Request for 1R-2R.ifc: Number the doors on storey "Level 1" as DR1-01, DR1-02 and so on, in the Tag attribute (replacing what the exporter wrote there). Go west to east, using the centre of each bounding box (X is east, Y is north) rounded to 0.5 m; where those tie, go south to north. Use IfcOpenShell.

First a look at what the model holds.

```python
import ifcopenshell
import ifcopenshell.util.element
import ifcopenshell.util.placement

model = ifcopenshell.open("1R-2R.ifc")
print(model.schema)
storey = next(s for s in model.by_type("IfcBuildingStorey") if s.Name == "Level 1")
doors = [e for e in ifcopenshell.util.element.get_decomposition(storey) if e.is_a("IfcDoor")]
for e in sorted(doors, key=lambda e: e.id()):
    origin = ifcopenshell.util.placement.get_local_placement(e.ObjectPlacement)[:3, 3]
    print(e.id(), e.Tag, e.Name, origin.round(2) + 0.0, sep=" | ")
```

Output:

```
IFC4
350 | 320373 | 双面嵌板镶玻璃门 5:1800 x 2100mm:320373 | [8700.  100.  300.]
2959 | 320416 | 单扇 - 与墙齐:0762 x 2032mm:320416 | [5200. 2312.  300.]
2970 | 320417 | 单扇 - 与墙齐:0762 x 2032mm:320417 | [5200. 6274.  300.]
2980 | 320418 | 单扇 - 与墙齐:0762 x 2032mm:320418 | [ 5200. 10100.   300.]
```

```python
import ifcopenshell
import ifcopenshell.geom
import ifcopenshell.util.element
import ifcopenshell.util.shape

model = ifcopenshell.open("1R-2R.ifc")
settings = ifcopenshell.geom.settings()
settings.set("use-world-coords", True)


def centre(element):
    shape = ifcopenshell.geom.create_shape(settings, element)
    return ifcopenshell.util.shape.get_bbox_centroid(shape.geometry)


storey = next(s for s in model.by_type("IfcBuildingStorey") if s.Name == "Level 1")
doors = [e for e in ifcopenshell.util.element.get_decomposition(storey) if e.is_a("IfcDoor")]

# Insertion points can sit at a corner or the storey origin, so sort by the geometry (in metres).
centres = {e: centre(e) for e in doors}
doors.sort(key=lambda e: (round(centres[e][0] / 0.5), centres[e][1]))

for i, e in enumerate(doors, start=1):
    number = f"DR1-{i:02d}"
    e.Tag = number
    print(e.id(), number)

model.write("1R-2R_updated.ifc")
```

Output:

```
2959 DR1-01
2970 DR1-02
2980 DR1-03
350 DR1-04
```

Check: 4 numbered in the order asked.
